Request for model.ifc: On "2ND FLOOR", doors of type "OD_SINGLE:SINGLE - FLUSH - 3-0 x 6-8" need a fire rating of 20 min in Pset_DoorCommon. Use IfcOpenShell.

First a look at what the model holds.

```python
import ifcopenshell
import ifcopenshell.util.element

model = ifcopenshell.open("model.ifc")
print(model.schema)
storey = next(s for s in model.by_type("IfcBuildingStorey") if s.Name == "2ND FLOOR")
doors = [e for e in ifcopenshell.util.element.get_decomposition(storey) if e.is_a("IfcDoor")]
seen = {}
for e in doors:
    element_type = ifcopenshell.util.element.get_type(e)
    key = (element_type.Name if element_type != e and element_type else None, ifcopenshell.util.element.get_pset(e, "Pset_DoorCommon", "FireRating"))
    seen[key] = seen.get(key, 0) + 1
for (name, value), count in sorted(seen.items(), key=str):
    print(count, "x", name, "|", value)
```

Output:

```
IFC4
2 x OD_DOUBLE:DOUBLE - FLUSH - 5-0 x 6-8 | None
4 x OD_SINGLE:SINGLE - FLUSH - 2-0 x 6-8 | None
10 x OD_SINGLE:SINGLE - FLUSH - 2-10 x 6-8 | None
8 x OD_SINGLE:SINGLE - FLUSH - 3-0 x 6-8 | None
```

```python
import ifcopenshell
import ifcopenshell.api.pset
import ifcopenshell.util.element

model = ifcopenshell.open("model.ifc")

storey = next(s for s in model.by_type("IfcBuildingStorey") if s.Name == "2ND FLOOR")
doors = [e for e in ifcopenshell.util.element.get_decomposition(storey) if e.is_a("IfcDoor")]

count = 0
for e in doors:
    element_type = ifcopenshell.util.element.get_type(e)
    if element_type in (None, e) or element_type.Name != "OD_SINGLE:SINGLE - FLUSH - 3-0 x 6-8":
        continue
    # add_pset returns the element's existing set when there is one.
    pset = ifcopenshell.api.pset.add_pset(model, product=e, name="Pset_DoorCommon")
    ifcopenshell.api.pset.edit_pset(model, pset=pset, properties={"FireRating": "20 min"})
    count += 1

print(count, "doors updated")

model.write("model_rev.ifc")
```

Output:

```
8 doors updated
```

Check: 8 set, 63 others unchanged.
